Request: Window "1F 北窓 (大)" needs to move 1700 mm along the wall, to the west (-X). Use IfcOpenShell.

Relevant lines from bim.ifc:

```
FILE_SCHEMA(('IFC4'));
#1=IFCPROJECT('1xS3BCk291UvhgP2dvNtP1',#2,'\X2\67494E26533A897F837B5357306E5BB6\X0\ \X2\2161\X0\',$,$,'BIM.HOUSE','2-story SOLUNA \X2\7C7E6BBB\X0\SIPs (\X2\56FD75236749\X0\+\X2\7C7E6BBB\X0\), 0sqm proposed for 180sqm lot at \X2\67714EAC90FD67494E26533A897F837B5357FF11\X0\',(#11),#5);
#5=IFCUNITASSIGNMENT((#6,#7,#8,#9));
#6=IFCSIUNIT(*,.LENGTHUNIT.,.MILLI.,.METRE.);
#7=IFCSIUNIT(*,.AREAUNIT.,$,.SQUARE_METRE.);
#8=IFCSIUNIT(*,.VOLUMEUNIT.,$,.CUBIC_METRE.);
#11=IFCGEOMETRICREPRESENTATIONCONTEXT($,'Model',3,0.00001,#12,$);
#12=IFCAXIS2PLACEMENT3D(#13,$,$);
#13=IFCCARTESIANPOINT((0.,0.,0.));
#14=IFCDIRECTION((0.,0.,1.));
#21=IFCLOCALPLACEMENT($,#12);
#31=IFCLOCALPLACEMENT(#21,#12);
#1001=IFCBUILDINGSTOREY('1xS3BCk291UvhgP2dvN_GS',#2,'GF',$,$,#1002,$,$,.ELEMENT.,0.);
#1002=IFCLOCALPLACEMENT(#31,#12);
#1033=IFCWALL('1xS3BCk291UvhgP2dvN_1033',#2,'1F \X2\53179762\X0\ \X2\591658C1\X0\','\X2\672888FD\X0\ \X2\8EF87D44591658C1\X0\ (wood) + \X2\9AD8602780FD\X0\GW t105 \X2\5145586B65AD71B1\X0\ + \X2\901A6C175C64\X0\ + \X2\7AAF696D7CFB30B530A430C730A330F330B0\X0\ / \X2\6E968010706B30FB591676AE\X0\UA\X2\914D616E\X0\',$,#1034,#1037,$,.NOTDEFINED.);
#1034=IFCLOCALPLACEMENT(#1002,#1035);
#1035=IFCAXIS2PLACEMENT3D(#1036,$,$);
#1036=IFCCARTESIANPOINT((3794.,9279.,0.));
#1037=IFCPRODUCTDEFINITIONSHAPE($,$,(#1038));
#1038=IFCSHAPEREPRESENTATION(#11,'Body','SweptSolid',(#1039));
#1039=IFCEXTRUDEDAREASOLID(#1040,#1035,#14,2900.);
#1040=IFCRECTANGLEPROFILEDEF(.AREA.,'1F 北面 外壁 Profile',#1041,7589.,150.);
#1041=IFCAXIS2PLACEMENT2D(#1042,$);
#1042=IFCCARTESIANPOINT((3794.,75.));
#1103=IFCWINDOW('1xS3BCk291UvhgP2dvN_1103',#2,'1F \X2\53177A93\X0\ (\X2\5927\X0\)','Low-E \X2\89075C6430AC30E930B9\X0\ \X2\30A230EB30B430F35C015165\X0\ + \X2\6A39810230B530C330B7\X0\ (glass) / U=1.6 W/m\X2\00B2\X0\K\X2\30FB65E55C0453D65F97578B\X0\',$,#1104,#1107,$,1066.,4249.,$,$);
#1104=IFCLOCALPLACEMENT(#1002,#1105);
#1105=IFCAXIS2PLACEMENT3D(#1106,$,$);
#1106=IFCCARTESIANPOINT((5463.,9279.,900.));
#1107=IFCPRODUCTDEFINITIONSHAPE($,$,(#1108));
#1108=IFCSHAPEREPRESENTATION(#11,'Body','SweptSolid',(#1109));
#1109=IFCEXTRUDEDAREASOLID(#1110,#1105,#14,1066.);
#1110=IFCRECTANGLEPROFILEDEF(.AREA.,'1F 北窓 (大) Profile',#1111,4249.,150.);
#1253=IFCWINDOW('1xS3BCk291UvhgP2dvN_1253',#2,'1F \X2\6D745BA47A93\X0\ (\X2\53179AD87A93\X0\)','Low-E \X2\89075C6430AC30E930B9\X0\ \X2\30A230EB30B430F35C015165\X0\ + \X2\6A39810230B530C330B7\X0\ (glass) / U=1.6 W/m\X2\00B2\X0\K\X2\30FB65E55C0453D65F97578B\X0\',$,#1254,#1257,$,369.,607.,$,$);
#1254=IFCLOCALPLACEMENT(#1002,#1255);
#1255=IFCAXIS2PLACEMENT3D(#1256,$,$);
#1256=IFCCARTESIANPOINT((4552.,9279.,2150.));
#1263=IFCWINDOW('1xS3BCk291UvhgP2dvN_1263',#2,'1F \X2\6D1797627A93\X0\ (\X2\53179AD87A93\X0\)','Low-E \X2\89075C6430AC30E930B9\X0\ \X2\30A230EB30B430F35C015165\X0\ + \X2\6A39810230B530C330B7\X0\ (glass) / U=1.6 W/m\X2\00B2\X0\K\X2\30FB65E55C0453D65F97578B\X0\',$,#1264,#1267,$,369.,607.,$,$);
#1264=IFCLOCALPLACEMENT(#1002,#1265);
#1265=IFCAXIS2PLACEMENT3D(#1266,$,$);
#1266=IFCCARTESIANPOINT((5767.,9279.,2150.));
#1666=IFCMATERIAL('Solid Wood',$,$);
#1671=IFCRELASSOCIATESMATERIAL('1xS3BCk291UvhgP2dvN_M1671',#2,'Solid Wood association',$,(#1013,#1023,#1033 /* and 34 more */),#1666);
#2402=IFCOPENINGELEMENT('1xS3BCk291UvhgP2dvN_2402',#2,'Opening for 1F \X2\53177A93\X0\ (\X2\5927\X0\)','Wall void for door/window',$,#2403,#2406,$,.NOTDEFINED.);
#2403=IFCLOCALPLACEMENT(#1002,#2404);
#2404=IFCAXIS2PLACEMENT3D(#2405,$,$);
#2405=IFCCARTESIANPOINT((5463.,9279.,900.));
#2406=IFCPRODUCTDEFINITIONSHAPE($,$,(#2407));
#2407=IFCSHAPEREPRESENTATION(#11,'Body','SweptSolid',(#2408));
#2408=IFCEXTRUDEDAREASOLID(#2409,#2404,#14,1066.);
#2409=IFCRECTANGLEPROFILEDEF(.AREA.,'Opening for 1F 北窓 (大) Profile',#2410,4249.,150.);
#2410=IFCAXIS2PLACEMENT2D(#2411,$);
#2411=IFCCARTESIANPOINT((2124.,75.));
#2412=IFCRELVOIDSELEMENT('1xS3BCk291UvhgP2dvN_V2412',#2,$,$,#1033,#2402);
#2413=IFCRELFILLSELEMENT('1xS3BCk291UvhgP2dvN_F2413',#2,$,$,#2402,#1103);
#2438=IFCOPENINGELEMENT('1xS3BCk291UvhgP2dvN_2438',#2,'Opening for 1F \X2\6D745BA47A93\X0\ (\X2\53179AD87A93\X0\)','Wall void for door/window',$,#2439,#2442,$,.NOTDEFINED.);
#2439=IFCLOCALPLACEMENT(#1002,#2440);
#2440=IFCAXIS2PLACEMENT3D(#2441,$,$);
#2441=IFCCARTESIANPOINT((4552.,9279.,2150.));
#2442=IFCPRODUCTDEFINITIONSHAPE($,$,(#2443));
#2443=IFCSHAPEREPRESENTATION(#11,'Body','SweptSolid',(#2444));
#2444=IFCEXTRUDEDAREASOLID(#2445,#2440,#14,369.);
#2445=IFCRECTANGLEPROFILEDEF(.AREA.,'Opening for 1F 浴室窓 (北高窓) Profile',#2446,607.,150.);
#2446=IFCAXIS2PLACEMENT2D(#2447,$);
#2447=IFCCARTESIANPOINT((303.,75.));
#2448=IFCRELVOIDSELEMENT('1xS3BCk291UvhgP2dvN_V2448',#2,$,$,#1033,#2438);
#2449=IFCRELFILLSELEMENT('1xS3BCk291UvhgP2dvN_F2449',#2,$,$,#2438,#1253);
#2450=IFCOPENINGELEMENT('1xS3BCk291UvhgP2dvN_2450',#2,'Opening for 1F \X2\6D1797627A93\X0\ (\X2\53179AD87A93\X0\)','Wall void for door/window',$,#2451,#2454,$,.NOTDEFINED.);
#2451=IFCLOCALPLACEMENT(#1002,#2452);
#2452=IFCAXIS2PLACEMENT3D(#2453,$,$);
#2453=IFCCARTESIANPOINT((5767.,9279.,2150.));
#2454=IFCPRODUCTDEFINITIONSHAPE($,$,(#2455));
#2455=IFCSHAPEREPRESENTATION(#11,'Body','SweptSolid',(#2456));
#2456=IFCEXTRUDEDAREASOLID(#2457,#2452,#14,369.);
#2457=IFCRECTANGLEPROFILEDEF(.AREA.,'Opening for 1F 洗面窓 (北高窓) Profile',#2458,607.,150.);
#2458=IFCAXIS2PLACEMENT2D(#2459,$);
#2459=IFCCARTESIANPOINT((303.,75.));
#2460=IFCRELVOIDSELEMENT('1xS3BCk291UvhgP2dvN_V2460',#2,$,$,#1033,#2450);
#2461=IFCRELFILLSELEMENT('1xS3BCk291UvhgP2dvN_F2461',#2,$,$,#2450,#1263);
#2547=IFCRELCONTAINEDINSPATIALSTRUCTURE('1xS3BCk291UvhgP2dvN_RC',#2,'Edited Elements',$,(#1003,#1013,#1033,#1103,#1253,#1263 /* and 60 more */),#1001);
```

```python
import ifcopenshell
import ifcopenshell.api.geometry
import ifcopenshell.util.placement
import ifcopenshell.util.unit

model = ifcopenshell.open("bim.ifc")
unit_scale = ifcopenshell.util.unit.calculate_unit_scale(model)

window = model.by_guid("1xS3BCk291UvhgP2dvN_1103")
opening = window.FillsVoids[0].RelatingOpeningElement
wall = opening.VoidsElements[0].RelatingBuildingElement

wall_matrix = ifcopenshell.util.placement.get_local_placement(wall.ObjectPlacement)
shift = wall_matrix[:3, 0] * -1.7 / unit_scale
before = ifcopenshell.util.placement.get_local_placement(window.ObjectPlacement)[:3, 3].copy()

# The window is not placed relative to its opening, so move both.
for product in (opening, window):
    matrix = ifcopenshell.util.placement.get_local_placement(product.ObjectPlacement)
    matrix[:3, 3] += shift
    ifcopenshell.api.geometry.edit_object_placement(model, product=product, matrix=matrix, is_si=False)

after = ifcopenshell.util.placement.get_local_placement(window.ObjectPlacement)[:3, 3]
print("window moved by", (after - before).round(3) + 0.0)

model.write("bim_v2.ifc")
```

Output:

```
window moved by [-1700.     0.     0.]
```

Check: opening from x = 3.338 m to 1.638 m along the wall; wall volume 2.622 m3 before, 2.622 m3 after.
